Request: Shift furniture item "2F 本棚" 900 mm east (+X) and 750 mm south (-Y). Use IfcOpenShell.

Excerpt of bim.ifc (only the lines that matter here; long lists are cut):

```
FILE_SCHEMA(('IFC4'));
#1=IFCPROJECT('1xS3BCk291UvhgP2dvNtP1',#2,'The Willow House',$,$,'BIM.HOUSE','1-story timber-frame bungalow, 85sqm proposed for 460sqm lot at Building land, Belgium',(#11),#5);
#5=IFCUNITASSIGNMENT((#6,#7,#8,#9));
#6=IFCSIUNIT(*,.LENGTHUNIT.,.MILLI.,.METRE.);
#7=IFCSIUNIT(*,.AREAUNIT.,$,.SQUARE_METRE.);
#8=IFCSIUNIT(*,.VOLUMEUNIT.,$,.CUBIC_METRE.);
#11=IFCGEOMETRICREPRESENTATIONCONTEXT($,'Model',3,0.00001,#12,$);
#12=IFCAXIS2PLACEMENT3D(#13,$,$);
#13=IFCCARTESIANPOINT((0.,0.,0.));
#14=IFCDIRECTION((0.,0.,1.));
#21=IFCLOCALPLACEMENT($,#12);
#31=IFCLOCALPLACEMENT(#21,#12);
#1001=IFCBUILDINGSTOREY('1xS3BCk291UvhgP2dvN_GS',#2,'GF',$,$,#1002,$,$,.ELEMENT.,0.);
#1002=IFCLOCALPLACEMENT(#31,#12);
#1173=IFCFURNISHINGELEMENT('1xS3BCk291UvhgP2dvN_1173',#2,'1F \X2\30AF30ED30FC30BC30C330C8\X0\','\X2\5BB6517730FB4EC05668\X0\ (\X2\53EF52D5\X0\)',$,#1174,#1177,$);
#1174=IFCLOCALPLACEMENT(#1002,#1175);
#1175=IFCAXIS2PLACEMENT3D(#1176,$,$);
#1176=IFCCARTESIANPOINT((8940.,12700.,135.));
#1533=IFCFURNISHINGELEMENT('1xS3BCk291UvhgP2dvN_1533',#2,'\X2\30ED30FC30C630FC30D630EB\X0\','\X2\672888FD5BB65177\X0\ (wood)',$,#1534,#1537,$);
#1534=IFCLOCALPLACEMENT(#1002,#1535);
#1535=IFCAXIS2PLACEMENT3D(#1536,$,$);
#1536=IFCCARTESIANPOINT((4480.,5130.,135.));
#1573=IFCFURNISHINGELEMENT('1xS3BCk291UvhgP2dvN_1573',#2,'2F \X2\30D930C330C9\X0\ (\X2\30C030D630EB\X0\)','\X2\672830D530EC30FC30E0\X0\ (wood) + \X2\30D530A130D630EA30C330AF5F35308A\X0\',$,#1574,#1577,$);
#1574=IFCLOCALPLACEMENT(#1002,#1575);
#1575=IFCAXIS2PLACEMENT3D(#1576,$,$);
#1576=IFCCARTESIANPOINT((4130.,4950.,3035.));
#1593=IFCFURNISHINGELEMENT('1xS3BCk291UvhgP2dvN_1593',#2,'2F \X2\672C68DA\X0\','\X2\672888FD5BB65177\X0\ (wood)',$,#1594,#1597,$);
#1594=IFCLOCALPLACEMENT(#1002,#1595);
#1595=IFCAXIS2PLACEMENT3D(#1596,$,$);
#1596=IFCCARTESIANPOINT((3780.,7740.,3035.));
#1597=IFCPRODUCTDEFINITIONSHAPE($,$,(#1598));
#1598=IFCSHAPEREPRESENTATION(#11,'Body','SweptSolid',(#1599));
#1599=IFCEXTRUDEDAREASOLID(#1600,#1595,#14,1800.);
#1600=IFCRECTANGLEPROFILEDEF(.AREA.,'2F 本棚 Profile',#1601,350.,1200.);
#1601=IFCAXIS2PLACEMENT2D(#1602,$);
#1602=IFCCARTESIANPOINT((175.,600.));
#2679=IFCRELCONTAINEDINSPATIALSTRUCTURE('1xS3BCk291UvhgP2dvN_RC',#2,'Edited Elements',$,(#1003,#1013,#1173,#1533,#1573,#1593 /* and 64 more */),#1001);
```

```python
import ifcopenshell
import ifcopenshell.api.geometry
import ifcopenshell.util.placement

model = ifcopenshell.open("bim.ifc")

item = model.by_guid("1xS3BCk291UvhgP2dvN_1593")
matrix = ifcopenshell.util.placement.get_local_placement(item.ObjectPlacement)
matrix[0, 3] += 900.0
matrix[1, 3] -= 750.0
ifcopenshell.api.geometry.edit_object_placement(model, product=item, matrix=matrix, is_si=False)

print(ifcopenshell.util.placement.get_local_placement(item.ObjectPlacement).round(3) + 0.0)

model.write("bim-out.ifc")
```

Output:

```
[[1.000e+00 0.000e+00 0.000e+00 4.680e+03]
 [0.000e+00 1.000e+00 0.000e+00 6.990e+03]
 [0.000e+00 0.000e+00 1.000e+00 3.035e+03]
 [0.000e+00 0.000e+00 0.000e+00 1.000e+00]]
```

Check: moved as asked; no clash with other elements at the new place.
